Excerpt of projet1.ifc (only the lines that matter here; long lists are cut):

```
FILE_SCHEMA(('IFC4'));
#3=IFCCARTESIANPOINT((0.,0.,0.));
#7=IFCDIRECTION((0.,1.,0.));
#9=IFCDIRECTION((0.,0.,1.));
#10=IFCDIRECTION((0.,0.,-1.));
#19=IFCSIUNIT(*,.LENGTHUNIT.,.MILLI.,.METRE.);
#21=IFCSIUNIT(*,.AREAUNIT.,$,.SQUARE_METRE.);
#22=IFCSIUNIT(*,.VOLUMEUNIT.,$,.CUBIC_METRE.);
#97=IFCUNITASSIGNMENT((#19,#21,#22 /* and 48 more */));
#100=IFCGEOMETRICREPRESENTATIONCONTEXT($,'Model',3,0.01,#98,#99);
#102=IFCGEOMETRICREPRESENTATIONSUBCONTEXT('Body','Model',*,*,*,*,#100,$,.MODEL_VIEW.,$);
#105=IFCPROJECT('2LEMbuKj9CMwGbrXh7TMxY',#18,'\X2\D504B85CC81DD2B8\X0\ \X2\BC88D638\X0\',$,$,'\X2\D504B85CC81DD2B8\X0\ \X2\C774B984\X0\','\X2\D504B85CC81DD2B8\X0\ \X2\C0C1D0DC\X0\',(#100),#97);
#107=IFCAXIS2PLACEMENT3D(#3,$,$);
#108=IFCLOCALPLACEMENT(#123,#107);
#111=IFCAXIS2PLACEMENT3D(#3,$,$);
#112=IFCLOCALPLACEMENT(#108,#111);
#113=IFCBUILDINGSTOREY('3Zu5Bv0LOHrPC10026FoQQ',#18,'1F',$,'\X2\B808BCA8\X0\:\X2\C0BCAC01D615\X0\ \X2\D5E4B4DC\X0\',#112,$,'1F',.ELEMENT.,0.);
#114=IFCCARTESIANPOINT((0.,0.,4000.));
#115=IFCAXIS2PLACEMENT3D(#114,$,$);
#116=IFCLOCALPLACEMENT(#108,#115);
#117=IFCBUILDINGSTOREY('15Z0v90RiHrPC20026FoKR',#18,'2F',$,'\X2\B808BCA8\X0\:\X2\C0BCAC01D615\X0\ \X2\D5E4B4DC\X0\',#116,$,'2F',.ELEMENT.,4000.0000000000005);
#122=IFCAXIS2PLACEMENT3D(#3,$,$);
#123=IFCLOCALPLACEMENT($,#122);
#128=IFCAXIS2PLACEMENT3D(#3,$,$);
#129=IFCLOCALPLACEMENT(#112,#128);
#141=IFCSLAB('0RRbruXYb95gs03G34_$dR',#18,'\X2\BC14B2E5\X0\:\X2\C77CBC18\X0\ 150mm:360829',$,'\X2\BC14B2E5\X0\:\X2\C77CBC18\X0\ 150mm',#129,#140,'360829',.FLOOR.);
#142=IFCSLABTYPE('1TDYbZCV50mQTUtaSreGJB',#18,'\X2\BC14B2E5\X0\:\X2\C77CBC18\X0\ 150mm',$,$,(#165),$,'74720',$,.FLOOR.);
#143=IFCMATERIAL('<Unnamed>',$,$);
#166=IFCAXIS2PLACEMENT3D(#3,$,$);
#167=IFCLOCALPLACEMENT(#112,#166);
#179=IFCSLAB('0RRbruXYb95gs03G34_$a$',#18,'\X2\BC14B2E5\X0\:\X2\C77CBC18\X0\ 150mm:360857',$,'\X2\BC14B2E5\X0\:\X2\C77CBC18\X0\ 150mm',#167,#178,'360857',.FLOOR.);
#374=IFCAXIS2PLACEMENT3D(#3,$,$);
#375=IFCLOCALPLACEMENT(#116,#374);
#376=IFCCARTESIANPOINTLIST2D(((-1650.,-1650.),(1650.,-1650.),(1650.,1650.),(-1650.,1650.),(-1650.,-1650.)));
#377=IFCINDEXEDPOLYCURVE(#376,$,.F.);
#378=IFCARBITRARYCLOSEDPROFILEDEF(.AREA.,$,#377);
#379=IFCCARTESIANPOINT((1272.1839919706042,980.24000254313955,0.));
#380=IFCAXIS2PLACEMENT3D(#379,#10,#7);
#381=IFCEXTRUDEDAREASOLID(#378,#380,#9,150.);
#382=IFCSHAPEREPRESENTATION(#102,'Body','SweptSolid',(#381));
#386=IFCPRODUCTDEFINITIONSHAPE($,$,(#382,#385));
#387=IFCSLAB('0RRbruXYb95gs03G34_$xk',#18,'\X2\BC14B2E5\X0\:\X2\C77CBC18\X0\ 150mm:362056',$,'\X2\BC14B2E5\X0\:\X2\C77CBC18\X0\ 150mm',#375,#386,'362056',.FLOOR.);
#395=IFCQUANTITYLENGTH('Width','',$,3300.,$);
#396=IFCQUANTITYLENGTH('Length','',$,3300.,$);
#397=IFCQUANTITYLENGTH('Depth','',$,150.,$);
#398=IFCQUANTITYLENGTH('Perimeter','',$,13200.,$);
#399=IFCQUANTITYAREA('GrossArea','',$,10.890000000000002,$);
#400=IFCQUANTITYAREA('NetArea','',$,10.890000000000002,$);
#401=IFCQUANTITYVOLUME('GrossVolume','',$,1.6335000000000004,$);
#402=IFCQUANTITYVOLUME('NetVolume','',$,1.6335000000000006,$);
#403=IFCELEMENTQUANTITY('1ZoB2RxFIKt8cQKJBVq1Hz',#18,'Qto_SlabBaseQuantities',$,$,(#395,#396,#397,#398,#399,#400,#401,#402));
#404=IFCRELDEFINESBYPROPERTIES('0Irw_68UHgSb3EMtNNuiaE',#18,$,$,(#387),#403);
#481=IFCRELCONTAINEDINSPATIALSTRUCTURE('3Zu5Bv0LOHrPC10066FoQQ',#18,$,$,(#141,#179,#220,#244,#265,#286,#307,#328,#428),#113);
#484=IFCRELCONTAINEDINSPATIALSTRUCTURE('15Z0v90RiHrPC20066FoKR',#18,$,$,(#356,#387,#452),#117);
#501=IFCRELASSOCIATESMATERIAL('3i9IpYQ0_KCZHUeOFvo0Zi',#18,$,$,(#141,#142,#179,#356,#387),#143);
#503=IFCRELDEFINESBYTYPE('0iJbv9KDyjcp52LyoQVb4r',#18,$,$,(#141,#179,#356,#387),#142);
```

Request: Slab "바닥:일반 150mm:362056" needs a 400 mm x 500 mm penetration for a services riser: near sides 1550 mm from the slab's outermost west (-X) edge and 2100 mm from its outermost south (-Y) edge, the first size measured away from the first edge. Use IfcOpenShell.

```python
import numpy as np
import ifcopenshell
import ifcopenshell.api.feature
import ifcopenshell.api.geometry
import ifcopenshell.api.pset
import ifcopenshell.api.root
import ifcopenshell.geom
import ifcopenshell.util.element
import ifcopenshell.util.placement
import ifcopenshell.util.representation
import ifcopenshell.util.shape
import ifcopenshell.util.unit

model = ifcopenshell.open("projet1.ifc")
unit_scale = ifcopenshell.util.unit.calculate_unit_scale(model)
area_scale = ifcopenshell.util.unit.calculate_unit_scale(model, "AREAUNIT")
volume_scale = ifcopenshell.util.unit.calculate_unit_scale(model, "VOLUMEUNIT")
settings = ifcopenshell.geom.settings()


def volume(element):
    """Net volume in cubic metres, openings subtracted."""
    shape = ifcopenshell.geom.create_shape(settings, element)
    return ifcopenshell.util.shape.get_volume(shape.geometry)


slab = model.by_id(387)
before = volume(slab)

# Extent in the slab's own axes, in metres. The edges named are its -X and -Y sides.
slab_shape = ifcopenshell.geom.create_shape(settings, slab)
vertices = ifcopenshell.util.shape.get_vertices(slab_shape.geometry)
x_min, y_min, bottom = vertices.min(axis=0)
top = vertices[:, 2].max()

opening = ifcopenshell.api.root.create_entity(model, ifc_class="IfcOpeningElement", name="Services riser opening", predefined_type="OPENING")
context = ifcopenshell.util.representation.get_context(model, "Model", "Body", "MODEL_VIEW")
width, depth = 0.4, 0.5
outline = [(0.0, 0.0), (width, 0.0), (width, depth), (0.0, depth), (0.0, 0.0)]
# Overshoot both faces by 50 mm so the cut is clean.
shape = ifcopenshell.api.geometry.add_slab_representation(
    model, context=context, depth=top - bottom + 0.1, polyline=outline
)
ifcopenshell.api.geometry.assign_representation(model, product=opening, representation=shape)

matrix = ifcopenshell.util.placement.get_local_placement(slab.ObjectPlacement)
matrix[:, 3] = matrix @ np.append(np.array([x_min + 1.55, y_min + 2.1, bottom - 0.05]) / unit_scale, 1.0)
ifcopenshell.api.geometry.edit_object_placement(model, product=opening, matrix=matrix, is_si=False)
ifcopenshell.api.feature.add_feature(model, feature=opening, element=slab)

after = volume(slab)

# Update the slab's stored quantities.
qto = model.by_id(ifcopenshell.util.element.get_pset(slab, "Qto_SlabBaseQuantities", should_inherit=False)["id"])
ifcopenshell.api.pset.edit_qto(model, qto=qto, properties={
    "NetArea": after / (top - bottom) / area_scale,
    "NetVolume": after / volume_scale,
})

print(f"slab volume {before:.3f} -> {after:.3f} m3")

model.write("projet1_v2.ifc")
```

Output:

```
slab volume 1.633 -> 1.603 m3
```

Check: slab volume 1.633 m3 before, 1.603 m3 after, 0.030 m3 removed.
